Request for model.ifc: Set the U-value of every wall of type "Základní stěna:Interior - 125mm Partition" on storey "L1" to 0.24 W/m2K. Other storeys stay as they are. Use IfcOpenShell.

First a look at what the model holds.

```python
import ifcopenshell
import ifcopenshell.util.element

model = ifcopenshell.open("model.ifc")
print(model.schema)
storey = next(s for s in model.by_type("IfcBuildingStorey") if s.Name == "L1")
walls = [e for e in ifcopenshell.util.element.get_decomposition(storey) if e.is_a("IfcWall")]
seen = {}
for e in walls:
    element_type = ifcopenshell.util.element.get_type(e)
    key = (element_type.Name if element_type != e and element_type else None, ifcopenshell.util.element.get_pset(e, "Pset_WallCommon", "ThermalTransmittance"))
    seen[key] = seen.get(key, 0) + 1
for (name, value), count in sorted(seen.items(), key=str):
    print(count, "x", name, "|", value)
```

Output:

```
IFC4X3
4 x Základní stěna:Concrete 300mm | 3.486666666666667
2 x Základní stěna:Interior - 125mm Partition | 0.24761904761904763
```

```python
import ifcopenshell
import ifcopenshell.api.pset
import ifcopenshell.util.element

model = ifcopenshell.open("model.ifc")

storey = next(s for s in model.by_type("IfcBuildingStorey") if s.Name == "L1")
walls = [e for e in ifcopenshell.util.element.get_decomposition(storey) if e.is_a("IfcWall")]

count = 0
for e in walls:
    element_type = ifcopenshell.util.element.get_type(e)
    if element_type in (None, e) or element_type.Name != "Základní stěna:Interior - 125mm Partition":
        continue
    # add_pset returns the element's existing set when there is one.
    pset = ifcopenshell.api.pset.add_pset(model, product=e, name="Pset_WallCommon")
    ifcopenshell.api.pset.edit_pset(model, pset=pset, properties={"ThermalTransmittance": 0.24})
    count += 1

print(count, "walls updated")

model.write("model_v2.ifc")
```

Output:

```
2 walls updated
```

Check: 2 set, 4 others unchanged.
